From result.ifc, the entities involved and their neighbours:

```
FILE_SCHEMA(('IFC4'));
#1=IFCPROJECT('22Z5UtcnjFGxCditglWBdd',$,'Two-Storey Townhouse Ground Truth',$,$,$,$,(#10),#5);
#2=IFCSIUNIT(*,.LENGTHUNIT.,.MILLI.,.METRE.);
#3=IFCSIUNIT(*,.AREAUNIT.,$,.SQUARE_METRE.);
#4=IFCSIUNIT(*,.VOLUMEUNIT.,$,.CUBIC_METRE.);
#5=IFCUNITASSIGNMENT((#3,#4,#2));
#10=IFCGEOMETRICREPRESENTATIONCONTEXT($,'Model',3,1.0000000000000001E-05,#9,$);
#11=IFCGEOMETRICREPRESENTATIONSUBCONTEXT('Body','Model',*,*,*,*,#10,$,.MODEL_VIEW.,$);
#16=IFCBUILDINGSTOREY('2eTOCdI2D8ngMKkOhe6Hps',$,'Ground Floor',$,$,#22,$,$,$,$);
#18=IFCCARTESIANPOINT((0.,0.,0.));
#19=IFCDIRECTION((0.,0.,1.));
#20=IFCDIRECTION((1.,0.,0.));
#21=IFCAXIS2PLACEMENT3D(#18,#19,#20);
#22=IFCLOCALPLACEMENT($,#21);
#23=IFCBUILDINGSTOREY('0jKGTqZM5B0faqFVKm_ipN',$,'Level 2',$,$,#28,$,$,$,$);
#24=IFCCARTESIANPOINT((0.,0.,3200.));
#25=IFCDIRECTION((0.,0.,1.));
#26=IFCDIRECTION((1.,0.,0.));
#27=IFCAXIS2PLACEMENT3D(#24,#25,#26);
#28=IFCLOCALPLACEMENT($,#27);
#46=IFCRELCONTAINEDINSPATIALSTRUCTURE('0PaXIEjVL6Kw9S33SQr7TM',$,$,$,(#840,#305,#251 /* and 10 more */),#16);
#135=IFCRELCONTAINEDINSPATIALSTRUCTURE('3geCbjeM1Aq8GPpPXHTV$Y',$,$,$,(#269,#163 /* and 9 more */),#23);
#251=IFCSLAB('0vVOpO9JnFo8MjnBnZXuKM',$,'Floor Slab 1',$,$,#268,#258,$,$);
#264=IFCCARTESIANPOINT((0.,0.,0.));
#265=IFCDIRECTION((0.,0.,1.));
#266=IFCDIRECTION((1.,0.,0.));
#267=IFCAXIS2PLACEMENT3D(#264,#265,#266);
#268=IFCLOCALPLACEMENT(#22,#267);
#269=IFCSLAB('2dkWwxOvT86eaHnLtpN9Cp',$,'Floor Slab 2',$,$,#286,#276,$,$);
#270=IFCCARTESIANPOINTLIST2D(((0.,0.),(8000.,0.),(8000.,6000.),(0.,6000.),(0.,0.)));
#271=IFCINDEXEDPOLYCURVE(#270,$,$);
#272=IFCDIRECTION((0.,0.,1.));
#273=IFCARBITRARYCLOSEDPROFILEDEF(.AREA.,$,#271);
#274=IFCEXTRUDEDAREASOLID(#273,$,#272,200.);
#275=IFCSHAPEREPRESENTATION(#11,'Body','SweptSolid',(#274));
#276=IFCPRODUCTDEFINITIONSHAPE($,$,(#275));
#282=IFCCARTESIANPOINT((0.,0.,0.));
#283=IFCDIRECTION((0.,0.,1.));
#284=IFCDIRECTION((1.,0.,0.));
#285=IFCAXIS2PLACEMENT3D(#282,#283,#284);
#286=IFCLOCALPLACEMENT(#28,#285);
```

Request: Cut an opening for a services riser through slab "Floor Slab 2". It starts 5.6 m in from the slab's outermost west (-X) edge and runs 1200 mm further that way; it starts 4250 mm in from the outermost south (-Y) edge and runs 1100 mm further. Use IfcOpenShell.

```python
import numpy as np
import ifcopenshell
import ifcopenshell.api.feature
import ifcopenshell.api.geometry
import ifcopenshell.api.root
import ifcopenshell.geom
import ifcopenshell.util.placement
import ifcopenshell.util.representation
import ifcopenshell.util.shape
import ifcopenshell.util.unit

model = ifcopenshell.open("result.ifc")
unit_scale = ifcopenshell.util.unit.calculate_unit_scale(model)
settings = ifcopenshell.geom.settings()


def volume(element):
    """Net volume in cubic metres, openings subtracted."""
    shape = ifcopenshell.geom.create_shape(settings, element)
    return ifcopenshell.util.shape.get_volume(shape.geometry)


slab = model.by_guid("2dkWwxOvT86eaHnLtpN9Cp")
before = volume(slab)

# Extent in the slab's own axes, in metres. The edges named are its -X and -Y sides.
slab_shape = ifcopenshell.geom.create_shape(settings, slab)
vertices = ifcopenshell.util.shape.get_vertices(slab_shape.geometry)
x_min, y_min, bottom = vertices.min(axis=0)
top = vertices[:, 2].max()

opening = ifcopenshell.api.root.create_entity(model, ifc_class="IfcOpeningElement", name="Services riser opening", predefined_type="OPENING")
context = ifcopenshell.util.representation.get_context(model, "Model", "Body", "MODEL_VIEW")
width, depth = 1.2, 1.1
outline = [(0.0, 0.0), (width, 0.0), (width, depth), (0.0, depth), (0.0, 0.0)]
# Overshoot both faces by 50 mm so the cut is clean.
shape = ifcopenshell.api.geometry.add_slab_representation(
    model, context=context, depth=top - bottom + 0.1, polyline=outline
)
ifcopenshell.api.geometry.assign_representation(model, product=opening, representation=shape)

matrix = ifcopenshell.util.placement.get_local_placement(slab.ObjectPlacement)
matrix[:, 3] = matrix @ np.append(np.array([x_min + 5.6, y_min + 4.25, bottom - 0.05]) / unit_scale, 1.0)
ifcopenshell.api.geometry.edit_object_placement(model, product=opening, matrix=matrix, is_si=False)
ifcopenshell.api.feature.add_feature(model, feature=opening, element=slab)

after = volume(slab)

print(f"slab volume {before:.3f} -> {after:.3f} m3")

model.write("result-out.ifc")
```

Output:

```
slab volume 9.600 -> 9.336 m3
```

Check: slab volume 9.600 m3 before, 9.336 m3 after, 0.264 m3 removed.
